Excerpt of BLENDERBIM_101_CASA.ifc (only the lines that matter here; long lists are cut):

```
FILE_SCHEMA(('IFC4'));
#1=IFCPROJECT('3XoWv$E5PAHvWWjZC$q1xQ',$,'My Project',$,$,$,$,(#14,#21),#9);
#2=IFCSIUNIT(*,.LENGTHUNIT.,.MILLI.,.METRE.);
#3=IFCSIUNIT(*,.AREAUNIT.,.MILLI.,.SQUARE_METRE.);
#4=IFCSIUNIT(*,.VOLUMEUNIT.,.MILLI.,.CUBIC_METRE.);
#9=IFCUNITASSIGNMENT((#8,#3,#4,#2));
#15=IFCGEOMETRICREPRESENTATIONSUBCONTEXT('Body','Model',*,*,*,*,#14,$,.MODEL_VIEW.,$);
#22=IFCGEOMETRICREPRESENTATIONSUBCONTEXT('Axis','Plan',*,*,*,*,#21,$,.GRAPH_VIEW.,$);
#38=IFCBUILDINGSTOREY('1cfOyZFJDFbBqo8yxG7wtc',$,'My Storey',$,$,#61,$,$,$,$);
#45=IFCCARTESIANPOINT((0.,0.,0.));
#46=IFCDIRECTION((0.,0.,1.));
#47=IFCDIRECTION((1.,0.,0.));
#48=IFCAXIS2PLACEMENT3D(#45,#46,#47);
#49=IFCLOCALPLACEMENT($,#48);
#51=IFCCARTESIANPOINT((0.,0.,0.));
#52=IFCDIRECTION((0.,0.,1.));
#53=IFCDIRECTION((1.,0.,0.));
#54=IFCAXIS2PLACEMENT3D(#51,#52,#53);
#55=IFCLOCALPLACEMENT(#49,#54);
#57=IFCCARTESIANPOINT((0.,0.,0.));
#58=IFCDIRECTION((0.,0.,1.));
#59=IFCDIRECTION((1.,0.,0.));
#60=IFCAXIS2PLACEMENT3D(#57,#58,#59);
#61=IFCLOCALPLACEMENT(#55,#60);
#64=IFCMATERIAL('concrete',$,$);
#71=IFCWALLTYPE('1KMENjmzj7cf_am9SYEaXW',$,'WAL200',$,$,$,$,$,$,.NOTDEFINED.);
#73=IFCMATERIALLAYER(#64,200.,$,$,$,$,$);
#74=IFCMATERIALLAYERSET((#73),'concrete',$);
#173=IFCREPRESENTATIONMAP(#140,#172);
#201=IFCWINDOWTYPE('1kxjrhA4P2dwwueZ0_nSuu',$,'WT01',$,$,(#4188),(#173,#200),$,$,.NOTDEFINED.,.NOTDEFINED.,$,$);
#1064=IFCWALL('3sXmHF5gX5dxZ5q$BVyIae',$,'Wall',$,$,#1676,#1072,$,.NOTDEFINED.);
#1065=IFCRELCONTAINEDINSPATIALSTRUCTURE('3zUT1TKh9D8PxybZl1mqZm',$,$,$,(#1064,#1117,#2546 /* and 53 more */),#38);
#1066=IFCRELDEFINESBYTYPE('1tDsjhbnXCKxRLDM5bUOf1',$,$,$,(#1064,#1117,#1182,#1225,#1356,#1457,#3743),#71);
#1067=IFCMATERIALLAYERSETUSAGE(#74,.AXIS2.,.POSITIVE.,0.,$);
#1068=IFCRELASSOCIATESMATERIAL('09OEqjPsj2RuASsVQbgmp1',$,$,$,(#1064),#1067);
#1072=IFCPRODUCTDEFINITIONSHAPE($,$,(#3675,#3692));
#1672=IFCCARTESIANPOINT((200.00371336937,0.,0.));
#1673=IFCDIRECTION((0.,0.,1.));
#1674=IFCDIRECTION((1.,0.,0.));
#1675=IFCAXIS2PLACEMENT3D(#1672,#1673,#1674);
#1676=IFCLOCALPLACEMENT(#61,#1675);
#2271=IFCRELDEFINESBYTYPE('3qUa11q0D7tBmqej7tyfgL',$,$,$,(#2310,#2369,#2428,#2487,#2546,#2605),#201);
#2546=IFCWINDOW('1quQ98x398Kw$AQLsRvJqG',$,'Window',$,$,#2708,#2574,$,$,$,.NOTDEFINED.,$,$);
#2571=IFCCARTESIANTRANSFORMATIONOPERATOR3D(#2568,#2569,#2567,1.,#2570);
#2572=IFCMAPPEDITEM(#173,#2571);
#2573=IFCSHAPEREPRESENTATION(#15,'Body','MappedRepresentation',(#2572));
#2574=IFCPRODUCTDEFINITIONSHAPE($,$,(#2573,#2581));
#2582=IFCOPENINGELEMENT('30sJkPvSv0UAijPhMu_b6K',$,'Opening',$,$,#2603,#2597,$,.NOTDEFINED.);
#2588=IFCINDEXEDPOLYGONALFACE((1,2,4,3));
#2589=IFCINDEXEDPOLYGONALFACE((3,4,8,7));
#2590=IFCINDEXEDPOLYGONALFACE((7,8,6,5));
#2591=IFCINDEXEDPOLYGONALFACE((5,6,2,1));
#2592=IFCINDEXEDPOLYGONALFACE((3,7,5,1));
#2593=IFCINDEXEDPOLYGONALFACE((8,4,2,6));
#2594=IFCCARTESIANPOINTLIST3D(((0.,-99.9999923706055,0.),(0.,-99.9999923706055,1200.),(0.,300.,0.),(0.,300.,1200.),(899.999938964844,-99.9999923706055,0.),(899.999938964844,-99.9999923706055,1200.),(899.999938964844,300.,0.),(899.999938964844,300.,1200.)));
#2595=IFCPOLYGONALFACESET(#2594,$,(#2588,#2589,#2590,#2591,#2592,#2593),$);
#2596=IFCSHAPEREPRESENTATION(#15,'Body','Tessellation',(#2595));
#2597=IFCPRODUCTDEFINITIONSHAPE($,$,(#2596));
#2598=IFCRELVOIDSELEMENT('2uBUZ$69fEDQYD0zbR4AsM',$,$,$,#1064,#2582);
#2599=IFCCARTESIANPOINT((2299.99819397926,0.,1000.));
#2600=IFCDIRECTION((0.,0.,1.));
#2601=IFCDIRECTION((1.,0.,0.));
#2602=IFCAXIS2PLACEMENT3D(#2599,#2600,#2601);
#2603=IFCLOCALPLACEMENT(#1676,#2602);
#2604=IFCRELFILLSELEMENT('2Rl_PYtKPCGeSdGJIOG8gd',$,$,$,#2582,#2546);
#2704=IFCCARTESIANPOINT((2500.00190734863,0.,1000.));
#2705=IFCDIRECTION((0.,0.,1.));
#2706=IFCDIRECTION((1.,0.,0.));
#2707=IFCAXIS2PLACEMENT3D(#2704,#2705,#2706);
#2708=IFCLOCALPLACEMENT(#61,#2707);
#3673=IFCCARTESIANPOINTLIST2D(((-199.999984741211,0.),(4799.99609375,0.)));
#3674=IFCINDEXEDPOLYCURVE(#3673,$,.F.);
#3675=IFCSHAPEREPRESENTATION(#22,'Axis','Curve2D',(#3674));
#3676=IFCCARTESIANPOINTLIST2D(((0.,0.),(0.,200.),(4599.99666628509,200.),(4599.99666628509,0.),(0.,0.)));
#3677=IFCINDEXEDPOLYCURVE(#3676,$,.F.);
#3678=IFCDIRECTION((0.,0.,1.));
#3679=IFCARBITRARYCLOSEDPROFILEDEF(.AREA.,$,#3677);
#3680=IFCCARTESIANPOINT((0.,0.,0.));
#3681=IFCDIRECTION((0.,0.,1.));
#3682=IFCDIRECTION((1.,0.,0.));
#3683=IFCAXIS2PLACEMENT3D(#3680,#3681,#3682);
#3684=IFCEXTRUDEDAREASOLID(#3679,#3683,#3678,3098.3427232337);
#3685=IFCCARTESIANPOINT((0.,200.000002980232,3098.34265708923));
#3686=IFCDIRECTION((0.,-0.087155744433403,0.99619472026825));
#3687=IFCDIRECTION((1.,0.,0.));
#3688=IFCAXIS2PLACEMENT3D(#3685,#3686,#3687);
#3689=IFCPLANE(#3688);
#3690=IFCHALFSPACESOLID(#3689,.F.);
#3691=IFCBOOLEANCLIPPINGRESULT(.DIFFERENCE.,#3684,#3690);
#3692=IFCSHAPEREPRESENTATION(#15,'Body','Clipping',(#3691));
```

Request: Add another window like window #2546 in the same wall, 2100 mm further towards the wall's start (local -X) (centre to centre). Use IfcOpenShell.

```python
import ifcopenshell
import ifcopenshell.api.feature
import ifcopenshell.api.geometry
import ifcopenshell.api.root
import ifcopenshell.geom
import ifcopenshell.util.element
import ifcopenshell.util.placement
import ifcopenshell.util.shape

model = ifcopenshell.open("BLENDERBIM_101_CASA.ifc")
settings = ifcopenshell.geom.settings()


def volume(element):
    """Net volume in cubic metres, openings subtracted."""
    shape = ifcopenshell.geom.create_shape(settings, element)
    return ifcopenshell.util.shape.get_volume(shape.geometry)


window = model.by_id(2546)
opening = window.FillsVoids[0].RelatingOpeningElement
wall = opening.VoidsElements[0].RelatingBuildingElement
before = volume(wall)
shift = ifcopenshell.util.placement.get_local_placement(wall.ObjectPlacement)[:3, 0] * -2100.0

# copy_class copies the void relationship, type, container and properties, but no geometry.
new_opening = ifcopenshell.api.root.copy_class(model, product=opening)
new_opening.Representation = ifcopenshell.util.element.copy_deep(
    model, opening.Representation, exclude=["IfcGeometricRepresentationContext", "IfcRepresentationMap"]
)
new_window = ifcopenshell.api.root.copy_class(model, product=window)
new_window.Representation = ifcopenshell.util.element.copy_deep(
    model, window.Representation, exclude=["IfcGeometricRepresentationContext", "IfcRepresentationMap"]
)
ifcopenshell.api.feature.add_filling(model, opening=new_opening, element=new_window)

for old, new in ((opening, new_opening), (window, new_window)):
    matrix = ifcopenshell.util.placement.get_local_placement(old.ObjectPlacement)
    matrix[:3, 3] += shift
    ifcopenshell.api.geometry.edit_object_placement(model, product=new, matrix=matrix, is_si=False)

after = volume(wall)

print(f"wall volume {before:.3f} -> {after:.3f} m3")

model.write("BLENDERBIM_101_CASA_v2.ifc")
```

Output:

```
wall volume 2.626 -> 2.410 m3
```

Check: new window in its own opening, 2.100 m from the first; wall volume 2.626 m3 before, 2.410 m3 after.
